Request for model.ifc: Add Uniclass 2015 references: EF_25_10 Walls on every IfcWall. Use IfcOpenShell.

First a look at what the model holds.

```python
import ifcopenshell

model = ifcopenshell.open("model.ifc")
print(model.schema)
print("classifications:", [c.Name for c in model.by_type("IfcClassification")])
for ifc_class in ("IfcDoor", "IfcRoof", "IfcStair", "IfcWall", "IfcWindow"):
    print(ifc_class, len(model.by_type(ifc_class)))
```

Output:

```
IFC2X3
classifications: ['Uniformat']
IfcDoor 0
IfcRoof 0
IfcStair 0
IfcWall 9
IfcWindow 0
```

```python
import ifcopenshell
import ifcopenshell.api.classification

model = ifcopenshell.open("model.ifc")

# IFC2X3 requires Source and Edition and has no link from the project to the system.
system = model.create_entity("IfcClassification", Source="NBS", Edition="2015", Name="Uniclass 2015")

codes = {
    "IfcWall": ("EF_25_10", "Walls"),
}
for ifc_class, (code, name) in codes.items():
    products = model.by_type(ifc_class)
    ifcopenshell.api.classification.add_reference(
        model, products=products, classification=system, identification=code, name=name
    )
    print(code, len(products))

model.write("model_v2.ifc")
```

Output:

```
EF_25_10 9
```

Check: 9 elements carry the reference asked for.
